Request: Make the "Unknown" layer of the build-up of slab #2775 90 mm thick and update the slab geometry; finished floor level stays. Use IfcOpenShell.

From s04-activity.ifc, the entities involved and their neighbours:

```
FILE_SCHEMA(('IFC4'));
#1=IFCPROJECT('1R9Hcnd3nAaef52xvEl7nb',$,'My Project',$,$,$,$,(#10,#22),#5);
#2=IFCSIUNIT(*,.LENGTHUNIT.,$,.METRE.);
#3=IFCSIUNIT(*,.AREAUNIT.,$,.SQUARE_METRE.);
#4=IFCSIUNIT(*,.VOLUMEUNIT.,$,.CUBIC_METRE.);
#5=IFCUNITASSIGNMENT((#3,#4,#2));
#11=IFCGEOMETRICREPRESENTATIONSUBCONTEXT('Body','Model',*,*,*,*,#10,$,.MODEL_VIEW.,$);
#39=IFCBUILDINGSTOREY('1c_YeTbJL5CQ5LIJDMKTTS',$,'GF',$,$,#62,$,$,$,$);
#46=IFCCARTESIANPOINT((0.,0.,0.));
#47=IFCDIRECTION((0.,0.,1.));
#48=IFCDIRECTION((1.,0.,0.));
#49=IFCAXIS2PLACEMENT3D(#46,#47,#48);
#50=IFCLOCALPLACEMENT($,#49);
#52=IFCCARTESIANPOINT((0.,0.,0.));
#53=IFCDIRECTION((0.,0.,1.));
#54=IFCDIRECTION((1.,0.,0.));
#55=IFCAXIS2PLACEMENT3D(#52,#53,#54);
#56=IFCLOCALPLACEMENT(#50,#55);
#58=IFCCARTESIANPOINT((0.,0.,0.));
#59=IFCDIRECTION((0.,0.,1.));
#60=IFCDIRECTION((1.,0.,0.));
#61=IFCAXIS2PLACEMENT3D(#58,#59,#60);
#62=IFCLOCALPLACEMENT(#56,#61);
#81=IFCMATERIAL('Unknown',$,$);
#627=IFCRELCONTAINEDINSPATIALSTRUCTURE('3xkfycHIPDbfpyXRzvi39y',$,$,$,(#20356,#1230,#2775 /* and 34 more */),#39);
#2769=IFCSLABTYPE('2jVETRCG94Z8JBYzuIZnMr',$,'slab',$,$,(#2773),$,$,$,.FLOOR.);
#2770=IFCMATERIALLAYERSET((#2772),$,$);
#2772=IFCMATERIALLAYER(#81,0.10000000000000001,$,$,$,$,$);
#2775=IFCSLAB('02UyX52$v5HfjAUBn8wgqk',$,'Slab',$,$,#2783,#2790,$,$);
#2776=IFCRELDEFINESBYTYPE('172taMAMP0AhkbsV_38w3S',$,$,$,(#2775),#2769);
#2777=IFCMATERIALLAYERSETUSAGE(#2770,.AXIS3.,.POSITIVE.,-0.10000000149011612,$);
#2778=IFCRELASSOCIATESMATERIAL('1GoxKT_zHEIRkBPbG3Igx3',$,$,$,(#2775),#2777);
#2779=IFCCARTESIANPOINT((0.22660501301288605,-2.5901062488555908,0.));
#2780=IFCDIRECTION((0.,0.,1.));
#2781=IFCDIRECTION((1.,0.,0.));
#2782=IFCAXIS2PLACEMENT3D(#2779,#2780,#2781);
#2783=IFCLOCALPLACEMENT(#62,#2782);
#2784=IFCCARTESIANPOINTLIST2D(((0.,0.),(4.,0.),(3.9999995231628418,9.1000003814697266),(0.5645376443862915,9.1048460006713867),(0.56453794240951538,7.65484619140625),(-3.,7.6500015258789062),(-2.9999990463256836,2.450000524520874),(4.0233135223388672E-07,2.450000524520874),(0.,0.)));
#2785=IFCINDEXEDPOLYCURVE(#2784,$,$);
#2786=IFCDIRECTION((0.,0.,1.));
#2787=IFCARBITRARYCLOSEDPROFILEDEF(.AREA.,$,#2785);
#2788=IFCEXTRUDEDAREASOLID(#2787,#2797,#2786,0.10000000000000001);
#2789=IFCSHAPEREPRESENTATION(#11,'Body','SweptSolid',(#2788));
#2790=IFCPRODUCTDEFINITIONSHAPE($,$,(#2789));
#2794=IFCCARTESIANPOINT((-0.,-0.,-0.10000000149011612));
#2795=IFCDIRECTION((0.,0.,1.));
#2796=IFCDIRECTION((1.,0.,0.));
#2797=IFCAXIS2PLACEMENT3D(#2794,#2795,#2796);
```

```python
import ifcopenshell
import ifcopenshell.util.element
import ifcopenshell.util.representation

model = ifcopenshell.open("s04-activity.ifc")

layer_set = model.by_id(2770)
layer = next(l for l in layer_set.MaterialLayers if l.Material and l.Material.Name == "Unknown")
change = 0.09 - layer.LayerThickness
layer.LayerThickness += change

# Geometry does not follow the layer set by itself.
slabs = [e for e in ifcopenshell.util.element.get_elements_by_material(model, layer_set) if e.is_a("IfcSlab")]
for slab in sorted(slabs, key=lambda e: e.id()):
    body = ifcopenshell.util.representation.get_representation(slab, "Model", "Body")
    solid = body.Items[0]
    old_depth = solid.Depth
    solid.Depth += change
    # Extruded upwards: lower the start of the extrusion so the top stays.
    x, y, z = solid.Position.Location.Coordinates
    solid.Position.Location = model.createIfcCartesianPoint((x, y, z - change))
    print(slab.id(), f"{old_depth:g} -> {solid.Depth:g}")

# The layers are counted up from the underside, which has moved.
for usage in {ifcopenshell.util.element.get_material(slab) for slab in slabs}:
    usage.OffsetFromReferenceLine -= change

model.write("s04-activity_v2.ifc")
```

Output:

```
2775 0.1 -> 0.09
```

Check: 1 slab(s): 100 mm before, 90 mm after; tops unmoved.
